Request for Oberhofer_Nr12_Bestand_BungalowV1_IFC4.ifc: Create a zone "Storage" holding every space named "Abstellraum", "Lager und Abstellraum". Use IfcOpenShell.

First a look at what the model holds.

```python
import ifcopenshell

model = ifcopenshell.open("Oberhofer_Nr12_Bestand_BungalowV1_IFC4.ifc")
print(model.schema)
seen = {}
for space in model.by_type("IfcSpace"):
    seen[space.LongName] = seen.get(space.LongName, 0) + 1
for name, count in sorted(seen.items(), key=str):
    print(count, "x", name)
print("zones:", [z.Name for z in model.by_type("IfcZone")][:20])
```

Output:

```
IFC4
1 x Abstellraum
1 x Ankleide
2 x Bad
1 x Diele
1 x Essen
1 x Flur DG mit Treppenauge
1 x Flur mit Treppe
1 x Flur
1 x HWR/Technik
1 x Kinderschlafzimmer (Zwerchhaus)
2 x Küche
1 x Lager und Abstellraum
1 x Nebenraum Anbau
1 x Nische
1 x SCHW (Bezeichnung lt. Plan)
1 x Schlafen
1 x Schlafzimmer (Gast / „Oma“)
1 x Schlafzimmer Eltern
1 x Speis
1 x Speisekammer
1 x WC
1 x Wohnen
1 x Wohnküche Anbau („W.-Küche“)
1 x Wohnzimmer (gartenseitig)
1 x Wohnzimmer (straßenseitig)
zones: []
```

```python
import ifcopenshell
import ifcopenshell.api.group
import ifcopenshell.api.root

model = ifcopenshell.open("Oberhofer_Nr12_Bestand_BungalowV1_IFC4.ifc")

names = {"Abstellraum", "Lager und Abstellraum"}
spaces = [s for s in model.by_type("IfcSpace") if s.LongName in names]

zone = ifcopenshell.api.root.create_entity(model, ifc_class="IfcZone", name="Storage")
ifcopenshell.api.group.assign_group(model, products=spaces, group=zone)
print(len(spaces), "spaces in", zone.Name)

model.write("Oberhofer_Nr12_Bestand_BungalowV1_IFC4_v2.ifc")
```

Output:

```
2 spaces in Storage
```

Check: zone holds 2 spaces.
